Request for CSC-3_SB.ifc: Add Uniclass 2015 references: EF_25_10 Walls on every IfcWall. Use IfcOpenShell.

First a look at what the model holds.

```python
import ifcopenshell

model = ifcopenshell.open("CSC-3_SB.ifc")
print(model.schema)
print("classifications:", [c.Name for c in model.by_type("IfcClassification")])
for ifc_class in ("IfcDoor", "IfcRoof", "IfcStair", "IfcWall", "IfcWindow"):
    print(ifc_class, len(model.by_type(ifc_class)))
```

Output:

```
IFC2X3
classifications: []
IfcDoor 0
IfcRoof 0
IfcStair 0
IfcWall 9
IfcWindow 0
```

```python
import ifcopenshell
import ifcopenshell.api.classification

model = ifcopenshell.open("CSC-3_SB.ifc")

# IFC2X3 requires Source and Edition and has no link from the project to the system.
system = model.create_entity("IfcClassification", Source="NBS", Edition="2015", Name="Uniclass 2015")

codes = {
    "IfcWall": ("EF_25_10", "Walls"),
}
for ifc_class, (code, name) in codes.items():
    products = model.by_type(ifc_class)
    ifcopenshell.api.classification.add_reference(
        model, products=products, classification=system, identification=code, name=name
    )
    print(code, len(products))

model.write("CSC-3_SB_rev.ifc")
```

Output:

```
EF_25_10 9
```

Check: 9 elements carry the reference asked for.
